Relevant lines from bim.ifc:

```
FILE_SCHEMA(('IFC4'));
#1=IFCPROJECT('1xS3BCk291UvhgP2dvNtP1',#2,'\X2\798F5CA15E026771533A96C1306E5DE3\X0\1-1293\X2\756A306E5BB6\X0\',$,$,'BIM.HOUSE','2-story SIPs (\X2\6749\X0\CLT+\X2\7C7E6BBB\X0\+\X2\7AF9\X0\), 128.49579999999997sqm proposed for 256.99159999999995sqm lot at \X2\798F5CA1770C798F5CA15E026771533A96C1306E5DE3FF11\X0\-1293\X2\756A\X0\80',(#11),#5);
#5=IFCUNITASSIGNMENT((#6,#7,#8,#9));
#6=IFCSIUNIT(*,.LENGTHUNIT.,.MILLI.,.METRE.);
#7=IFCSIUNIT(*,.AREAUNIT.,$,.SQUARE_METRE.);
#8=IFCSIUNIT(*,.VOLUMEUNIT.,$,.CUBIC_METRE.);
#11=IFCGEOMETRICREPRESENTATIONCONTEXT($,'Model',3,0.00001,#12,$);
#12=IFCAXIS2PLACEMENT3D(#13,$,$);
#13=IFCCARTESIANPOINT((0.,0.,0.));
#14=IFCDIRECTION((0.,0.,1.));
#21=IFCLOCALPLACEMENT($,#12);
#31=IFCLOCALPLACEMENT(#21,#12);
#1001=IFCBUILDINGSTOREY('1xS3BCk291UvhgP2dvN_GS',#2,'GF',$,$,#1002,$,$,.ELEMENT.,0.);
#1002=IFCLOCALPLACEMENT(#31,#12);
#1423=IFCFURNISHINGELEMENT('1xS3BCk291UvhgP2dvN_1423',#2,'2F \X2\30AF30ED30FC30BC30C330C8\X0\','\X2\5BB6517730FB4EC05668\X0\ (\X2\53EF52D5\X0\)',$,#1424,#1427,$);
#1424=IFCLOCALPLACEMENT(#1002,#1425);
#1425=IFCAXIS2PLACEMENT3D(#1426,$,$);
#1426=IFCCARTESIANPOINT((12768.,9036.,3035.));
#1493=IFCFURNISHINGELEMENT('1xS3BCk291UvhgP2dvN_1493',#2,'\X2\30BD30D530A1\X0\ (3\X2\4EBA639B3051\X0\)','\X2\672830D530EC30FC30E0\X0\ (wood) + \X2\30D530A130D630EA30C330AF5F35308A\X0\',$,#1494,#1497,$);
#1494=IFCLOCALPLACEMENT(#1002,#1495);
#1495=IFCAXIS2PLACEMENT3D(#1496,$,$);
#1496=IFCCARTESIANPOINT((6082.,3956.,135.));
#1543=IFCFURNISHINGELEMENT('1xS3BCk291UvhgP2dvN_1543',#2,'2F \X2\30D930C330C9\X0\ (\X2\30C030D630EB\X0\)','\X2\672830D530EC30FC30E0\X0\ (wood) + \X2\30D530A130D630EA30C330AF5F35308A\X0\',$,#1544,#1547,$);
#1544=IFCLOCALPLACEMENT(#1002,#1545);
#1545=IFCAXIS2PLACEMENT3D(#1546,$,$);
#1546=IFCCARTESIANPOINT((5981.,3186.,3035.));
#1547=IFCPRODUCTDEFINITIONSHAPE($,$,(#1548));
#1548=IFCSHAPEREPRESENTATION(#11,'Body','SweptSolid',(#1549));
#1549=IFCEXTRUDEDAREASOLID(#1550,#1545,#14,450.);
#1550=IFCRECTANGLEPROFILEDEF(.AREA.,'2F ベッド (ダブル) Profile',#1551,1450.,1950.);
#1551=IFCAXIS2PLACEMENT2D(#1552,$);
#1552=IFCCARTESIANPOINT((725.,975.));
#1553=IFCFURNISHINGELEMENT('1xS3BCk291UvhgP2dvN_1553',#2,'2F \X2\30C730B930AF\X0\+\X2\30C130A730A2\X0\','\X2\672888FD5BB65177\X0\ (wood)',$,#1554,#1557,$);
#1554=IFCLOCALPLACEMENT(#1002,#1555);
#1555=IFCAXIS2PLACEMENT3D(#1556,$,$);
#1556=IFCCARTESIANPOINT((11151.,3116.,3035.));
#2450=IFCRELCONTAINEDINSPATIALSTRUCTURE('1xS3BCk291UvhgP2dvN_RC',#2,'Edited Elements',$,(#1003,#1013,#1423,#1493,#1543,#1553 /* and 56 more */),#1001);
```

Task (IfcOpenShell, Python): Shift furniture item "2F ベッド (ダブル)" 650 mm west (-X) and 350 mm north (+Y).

```python
import ifcopenshell
import ifcopenshell.api.geometry
import ifcopenshell.util.placement
import ifcopenshell.util.unit

model = ifcopenshell.open("bim.ifc")
unit_scale = ifcopenshell.util.unit.calculate_unit_scale(model)

item = model.by_id(1543)
matrix = ifcopenshell.util.placement.get_local_placement(item.ObjectPlacement)
matrix[0, 3] -= 0.65 / unit_scale
matrix[1, 3] += 0.35 / unit_scale
ifcopenshell.api.geometry.edit_object_placement(model, product=item, matrix=matrix, is_si=False)

print(ifcopenshell.util.placement.get_local_placement(item.ObjectPlacement).round(3) + 0.0)

model.write("bim-out.ifc")
```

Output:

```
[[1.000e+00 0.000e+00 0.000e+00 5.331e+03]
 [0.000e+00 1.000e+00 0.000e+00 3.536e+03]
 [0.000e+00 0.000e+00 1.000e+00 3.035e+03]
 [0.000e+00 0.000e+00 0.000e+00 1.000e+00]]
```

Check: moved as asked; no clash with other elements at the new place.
